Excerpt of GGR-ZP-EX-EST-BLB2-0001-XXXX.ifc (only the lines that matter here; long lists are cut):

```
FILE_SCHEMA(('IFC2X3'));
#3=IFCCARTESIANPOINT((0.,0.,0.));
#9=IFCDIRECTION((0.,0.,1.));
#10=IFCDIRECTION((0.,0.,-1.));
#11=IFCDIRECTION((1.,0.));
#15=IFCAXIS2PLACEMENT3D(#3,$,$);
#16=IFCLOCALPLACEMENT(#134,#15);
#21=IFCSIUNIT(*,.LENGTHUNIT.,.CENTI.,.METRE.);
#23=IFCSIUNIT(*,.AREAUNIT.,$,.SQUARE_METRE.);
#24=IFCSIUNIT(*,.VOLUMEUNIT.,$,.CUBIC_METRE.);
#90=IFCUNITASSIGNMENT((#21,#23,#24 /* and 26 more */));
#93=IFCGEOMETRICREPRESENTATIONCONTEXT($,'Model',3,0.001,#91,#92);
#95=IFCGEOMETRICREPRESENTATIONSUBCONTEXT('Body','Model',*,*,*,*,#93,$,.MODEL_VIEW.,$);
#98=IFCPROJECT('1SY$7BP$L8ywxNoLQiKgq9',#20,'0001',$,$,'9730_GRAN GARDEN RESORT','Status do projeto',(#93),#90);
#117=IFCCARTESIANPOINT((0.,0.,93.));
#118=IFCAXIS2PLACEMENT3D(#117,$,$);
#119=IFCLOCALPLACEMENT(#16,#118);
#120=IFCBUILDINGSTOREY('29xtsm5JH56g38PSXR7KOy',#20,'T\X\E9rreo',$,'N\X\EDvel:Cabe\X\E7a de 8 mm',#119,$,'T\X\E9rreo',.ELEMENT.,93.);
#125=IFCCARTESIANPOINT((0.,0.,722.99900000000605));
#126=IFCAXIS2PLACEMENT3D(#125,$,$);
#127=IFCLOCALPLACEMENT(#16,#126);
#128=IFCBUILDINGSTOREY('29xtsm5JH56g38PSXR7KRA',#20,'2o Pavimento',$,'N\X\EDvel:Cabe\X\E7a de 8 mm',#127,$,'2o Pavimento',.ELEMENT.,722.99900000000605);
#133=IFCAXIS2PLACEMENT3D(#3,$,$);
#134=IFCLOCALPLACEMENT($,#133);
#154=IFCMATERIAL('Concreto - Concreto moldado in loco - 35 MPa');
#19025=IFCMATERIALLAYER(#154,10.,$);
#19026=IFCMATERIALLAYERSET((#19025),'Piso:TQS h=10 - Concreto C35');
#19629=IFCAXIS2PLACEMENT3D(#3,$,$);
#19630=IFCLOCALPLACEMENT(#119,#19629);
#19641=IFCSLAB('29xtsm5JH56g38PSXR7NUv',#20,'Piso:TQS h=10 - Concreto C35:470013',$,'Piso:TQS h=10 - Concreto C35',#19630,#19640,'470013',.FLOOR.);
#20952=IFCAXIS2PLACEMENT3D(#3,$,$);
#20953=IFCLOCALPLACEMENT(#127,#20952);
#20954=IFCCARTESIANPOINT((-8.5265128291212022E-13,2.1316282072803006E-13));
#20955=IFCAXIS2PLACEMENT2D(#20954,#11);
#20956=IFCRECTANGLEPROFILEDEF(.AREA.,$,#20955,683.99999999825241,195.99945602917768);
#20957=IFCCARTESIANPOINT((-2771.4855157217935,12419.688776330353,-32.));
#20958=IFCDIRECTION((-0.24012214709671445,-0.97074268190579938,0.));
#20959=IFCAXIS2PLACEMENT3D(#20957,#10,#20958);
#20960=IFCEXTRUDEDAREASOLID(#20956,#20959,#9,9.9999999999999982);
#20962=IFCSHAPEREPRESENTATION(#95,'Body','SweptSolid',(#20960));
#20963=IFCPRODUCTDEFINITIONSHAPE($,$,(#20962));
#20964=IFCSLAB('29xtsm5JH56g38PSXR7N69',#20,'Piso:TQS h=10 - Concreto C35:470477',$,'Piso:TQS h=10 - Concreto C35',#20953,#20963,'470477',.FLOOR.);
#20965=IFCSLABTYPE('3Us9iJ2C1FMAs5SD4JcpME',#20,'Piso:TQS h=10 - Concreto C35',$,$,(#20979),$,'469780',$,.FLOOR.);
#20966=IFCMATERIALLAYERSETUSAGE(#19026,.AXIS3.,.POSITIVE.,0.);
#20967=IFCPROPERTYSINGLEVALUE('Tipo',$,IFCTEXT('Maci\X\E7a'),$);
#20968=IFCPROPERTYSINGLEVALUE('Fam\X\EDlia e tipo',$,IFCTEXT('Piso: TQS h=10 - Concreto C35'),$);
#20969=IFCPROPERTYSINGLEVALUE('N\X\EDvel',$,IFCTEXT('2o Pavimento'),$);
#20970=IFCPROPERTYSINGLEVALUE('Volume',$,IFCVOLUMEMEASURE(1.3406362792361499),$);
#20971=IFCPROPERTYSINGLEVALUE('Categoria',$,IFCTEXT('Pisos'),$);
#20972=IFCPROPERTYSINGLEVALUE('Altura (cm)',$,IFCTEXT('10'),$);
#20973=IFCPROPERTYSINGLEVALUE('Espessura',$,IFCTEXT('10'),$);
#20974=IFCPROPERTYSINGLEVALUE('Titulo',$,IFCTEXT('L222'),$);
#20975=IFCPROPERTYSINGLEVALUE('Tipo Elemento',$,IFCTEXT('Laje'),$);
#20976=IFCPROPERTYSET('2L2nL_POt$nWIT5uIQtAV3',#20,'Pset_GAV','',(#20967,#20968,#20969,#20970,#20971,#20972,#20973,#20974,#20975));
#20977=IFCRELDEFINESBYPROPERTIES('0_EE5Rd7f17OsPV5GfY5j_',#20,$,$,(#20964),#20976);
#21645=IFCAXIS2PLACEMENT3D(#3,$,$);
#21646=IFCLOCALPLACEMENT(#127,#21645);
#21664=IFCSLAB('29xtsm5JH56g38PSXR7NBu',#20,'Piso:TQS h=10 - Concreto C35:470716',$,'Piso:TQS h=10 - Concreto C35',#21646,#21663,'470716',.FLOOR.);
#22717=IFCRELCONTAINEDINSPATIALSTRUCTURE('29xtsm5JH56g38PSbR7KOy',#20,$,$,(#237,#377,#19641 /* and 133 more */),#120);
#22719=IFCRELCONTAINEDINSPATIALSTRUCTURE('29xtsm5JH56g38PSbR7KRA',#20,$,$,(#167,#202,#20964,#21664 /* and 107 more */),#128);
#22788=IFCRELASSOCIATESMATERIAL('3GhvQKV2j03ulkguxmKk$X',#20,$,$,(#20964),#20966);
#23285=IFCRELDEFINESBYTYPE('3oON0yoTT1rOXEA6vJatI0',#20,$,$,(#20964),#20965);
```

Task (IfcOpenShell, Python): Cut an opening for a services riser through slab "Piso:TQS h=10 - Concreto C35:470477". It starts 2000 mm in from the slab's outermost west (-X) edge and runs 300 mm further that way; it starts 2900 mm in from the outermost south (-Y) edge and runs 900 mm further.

```python
import numpy as np
import ifcopenshell
import ifcopenshell.api.feature
import ifcopenshell.api.geometry
import ifcopenshell.api.pset
import ifcopenshell.api.root
import ifcopenshell.geom
import ifcopenshell.util.element
import ifcopenshell.util.placement
import ifcopenshell.util.representation
import ifcopenshell.util.shape
import ifcopenshell.util.unit

model = ifcopenshell.open("GGR-ZP-EX-EST-BLB2-0001-XXXX.ifc")
unit_scale = ifcopenshell.util.unit.calculate_unit_scale(model)
volume_scale = ifcopenshell.util.unit.calculate_unit_scale(model, "VOLUMEUNIT")
settings = ifcopenshell.geom.settings()


def volume(element):
    """Net volume in cubic metres, openings subtracted."""
    shape = ifcopenshell.geom.create_shape(settings, element)
    return ifcopenshell.util.shape.get_volume(shape.geometry)


slab = model.by_guid("29xtsm5JH56g38PSXR7N69")
before = volume(slab)

# Extent in the slab's own axes, in metres. The edges named are its -X and -Y sides.
slab_shape = ifcopenshell.geom.create_shape(settings, slab)
vertices = ifcopenshell.util.shape.get_vertices(slab_shape.geometry)
x_min, y_min, bottom = vertices.min(axis=0)
top = vertices[:, 2].max()

opening = ifcopenshell.api.root.create_entity(model, ifc_class="IfcOpeningElement", name="Services riser opening")
context = ifcopenshell.util.representation.get_context(model, "Model", "Body", "MODEL_VIEW")
width, depth = 0.3, 0.9
outline = [(0.0, 0.0), (width, 0.0), (width, depth), (0.0, depth), (0.0, 0.0)]
# Overshoot both faces by 50 mm so the cut is clean.
shape = ifcopenshell.api.geometry.add_slab_representation(
    model, context=context, depth=top - bottom + 0.1, polyline=outline
)
ifcopenshell.api.geometry.assign_representation(model, product=opening, representation=shape)

matrix = ifcopenshell.util.placement.get_local_placement(slab.ObjectPlacement)
matrix[:, 3] = matrix @ np.append(np.array([x_min + 2, y_min + 2.9, bottom - 0.05]) / unit_scale, 1.0)
ifcopenshell.api.geometry.edit_object_placement(model, product=opening, matrix=matrix, is_si=False)
ifcopenshell.api.feature.add_feature(model, feature=opening, element=slab)

after = volume(slab)

# Update the slab's stored quantities.
pset = model.by_id(ifcopenshell.util.element.get_pset(slab, "Pset_GAV", should_inherit=False)["id"])
ifcopenshell.api.pset.edit_pset(model, pset=pset, properties={
    "Volume": model.create_entity("IfcVolumeMeasure", after / volume_scale),
})

print(f"slab volume {before:.3f} -> {after:.3f} m3")

model.write("GGR-ZP-EX-EST-BLB2-0001-XXXX_updated.ifc")
```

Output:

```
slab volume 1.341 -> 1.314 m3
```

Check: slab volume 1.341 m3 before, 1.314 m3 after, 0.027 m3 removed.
